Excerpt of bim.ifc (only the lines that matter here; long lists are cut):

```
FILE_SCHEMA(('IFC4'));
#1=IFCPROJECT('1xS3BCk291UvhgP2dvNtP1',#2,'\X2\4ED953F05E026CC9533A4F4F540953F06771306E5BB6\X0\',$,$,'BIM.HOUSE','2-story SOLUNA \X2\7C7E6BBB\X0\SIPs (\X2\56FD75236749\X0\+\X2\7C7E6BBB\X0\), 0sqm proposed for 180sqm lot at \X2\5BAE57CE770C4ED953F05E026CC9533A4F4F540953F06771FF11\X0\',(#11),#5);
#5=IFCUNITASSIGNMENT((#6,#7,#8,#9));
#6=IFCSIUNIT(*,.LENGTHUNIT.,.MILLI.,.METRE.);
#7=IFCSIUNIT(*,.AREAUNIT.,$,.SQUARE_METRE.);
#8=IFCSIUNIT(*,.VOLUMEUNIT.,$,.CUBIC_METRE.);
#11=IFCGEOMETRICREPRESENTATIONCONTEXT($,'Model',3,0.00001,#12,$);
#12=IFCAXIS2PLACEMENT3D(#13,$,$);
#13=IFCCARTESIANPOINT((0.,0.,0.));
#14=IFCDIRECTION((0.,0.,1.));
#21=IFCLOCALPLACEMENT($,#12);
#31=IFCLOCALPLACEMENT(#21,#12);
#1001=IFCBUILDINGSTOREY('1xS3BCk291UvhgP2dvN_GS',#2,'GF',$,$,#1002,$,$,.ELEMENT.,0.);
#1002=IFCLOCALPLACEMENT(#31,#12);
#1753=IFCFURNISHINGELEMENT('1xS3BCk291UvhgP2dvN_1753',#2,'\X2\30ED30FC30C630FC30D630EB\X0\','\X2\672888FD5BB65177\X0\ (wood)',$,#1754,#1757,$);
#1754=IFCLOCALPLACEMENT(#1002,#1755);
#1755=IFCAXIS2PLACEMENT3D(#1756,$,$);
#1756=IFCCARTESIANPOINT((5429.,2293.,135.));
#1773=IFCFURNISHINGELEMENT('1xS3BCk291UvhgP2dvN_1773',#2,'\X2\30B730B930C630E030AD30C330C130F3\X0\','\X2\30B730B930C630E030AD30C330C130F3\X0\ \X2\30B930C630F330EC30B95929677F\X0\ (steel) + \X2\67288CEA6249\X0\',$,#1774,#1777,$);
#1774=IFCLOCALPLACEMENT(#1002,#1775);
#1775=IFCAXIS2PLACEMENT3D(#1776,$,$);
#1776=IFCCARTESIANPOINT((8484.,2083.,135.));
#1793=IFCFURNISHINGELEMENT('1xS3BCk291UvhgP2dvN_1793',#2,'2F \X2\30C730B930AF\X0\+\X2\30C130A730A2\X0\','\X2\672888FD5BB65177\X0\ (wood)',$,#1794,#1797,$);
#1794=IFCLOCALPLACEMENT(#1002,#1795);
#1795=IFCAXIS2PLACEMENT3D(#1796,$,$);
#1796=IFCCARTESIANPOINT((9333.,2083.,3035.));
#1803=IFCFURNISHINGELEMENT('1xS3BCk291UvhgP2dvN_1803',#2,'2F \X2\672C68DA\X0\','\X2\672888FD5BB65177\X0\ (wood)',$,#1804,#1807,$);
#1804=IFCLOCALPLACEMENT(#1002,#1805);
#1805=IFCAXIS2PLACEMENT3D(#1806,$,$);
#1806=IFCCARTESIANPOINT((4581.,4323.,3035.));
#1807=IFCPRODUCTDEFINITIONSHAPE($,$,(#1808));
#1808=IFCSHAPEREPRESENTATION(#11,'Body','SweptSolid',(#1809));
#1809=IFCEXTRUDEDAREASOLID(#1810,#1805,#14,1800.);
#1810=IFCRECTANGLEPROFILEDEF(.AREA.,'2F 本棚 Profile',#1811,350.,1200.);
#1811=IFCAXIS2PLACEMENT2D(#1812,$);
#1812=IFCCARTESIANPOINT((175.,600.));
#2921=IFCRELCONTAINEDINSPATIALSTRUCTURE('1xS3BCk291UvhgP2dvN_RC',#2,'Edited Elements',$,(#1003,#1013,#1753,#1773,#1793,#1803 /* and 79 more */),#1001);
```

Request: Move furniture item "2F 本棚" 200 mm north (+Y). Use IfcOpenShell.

```python
import ifcopenshell
import ifcopenshell.api.geometry
import ifcopenshell.util.placement

model = ifcopenshell.open("bim.ifc")

item = model.by_id(1803)
matrix = ifcopenshell.util.placement.get_local_placement(item.ObjectPlacement)
matrix[1, 3] += 200.0
ifcopenshell.api.geometry.edit_object_placement(model, product=item, matrix=matrix, is_si=False)

print(ifcopenshell.util.placement.get_local_placement(item.ObjectPlacement).round(3) + 0.0)

model.write("bim_v2.ifc")
```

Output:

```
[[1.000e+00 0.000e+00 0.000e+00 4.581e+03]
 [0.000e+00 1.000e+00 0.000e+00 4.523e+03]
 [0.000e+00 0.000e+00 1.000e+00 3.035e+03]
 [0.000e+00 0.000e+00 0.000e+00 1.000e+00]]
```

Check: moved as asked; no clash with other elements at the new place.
